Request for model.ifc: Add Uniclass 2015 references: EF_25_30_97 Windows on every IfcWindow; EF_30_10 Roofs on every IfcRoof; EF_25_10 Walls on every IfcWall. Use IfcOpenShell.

First a look at what the model holds.

```python
import ifcopenshell

model = ifcopenshell.open("model.ifc")
print(model.schema)
print("classifications:", [c.Name for c in model.by_type("IfcClassification")])
for ifc_class in ("IfcDoor", "IfcRoof", "IfcStair", "IfcWall", "IfcWindow"):
    print(ifc_class, len(model.by_type(ifc_class)))
```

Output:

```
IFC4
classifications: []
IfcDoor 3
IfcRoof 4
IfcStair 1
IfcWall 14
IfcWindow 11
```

```python
import ifcopenshell
import ifcopenshell.api.classification

model = ifcopenshell.open("model.ifc")

system = ifcopenshell.api.classification.add_classification(model, classification="Uniclass 2015")

codes = {
    "IfcWindow": ("EF_25_30_97", "Windows"),
    "IfcRoof": ("EF_30_10", "Roofs"),
    "IfcWall": ("EF_25_10", "Walls"),
}
for ifc_class, (code, name) in codes.items():
    products = model.by_type(ifc_class)
    ifcopenshell.api.classification.add_reference(
        model, products=products, classification=system, identification=code, name=name
    )
    print(code, len(products))

model.write("model_edited.ifc")
```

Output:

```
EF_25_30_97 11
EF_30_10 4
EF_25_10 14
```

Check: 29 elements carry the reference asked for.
